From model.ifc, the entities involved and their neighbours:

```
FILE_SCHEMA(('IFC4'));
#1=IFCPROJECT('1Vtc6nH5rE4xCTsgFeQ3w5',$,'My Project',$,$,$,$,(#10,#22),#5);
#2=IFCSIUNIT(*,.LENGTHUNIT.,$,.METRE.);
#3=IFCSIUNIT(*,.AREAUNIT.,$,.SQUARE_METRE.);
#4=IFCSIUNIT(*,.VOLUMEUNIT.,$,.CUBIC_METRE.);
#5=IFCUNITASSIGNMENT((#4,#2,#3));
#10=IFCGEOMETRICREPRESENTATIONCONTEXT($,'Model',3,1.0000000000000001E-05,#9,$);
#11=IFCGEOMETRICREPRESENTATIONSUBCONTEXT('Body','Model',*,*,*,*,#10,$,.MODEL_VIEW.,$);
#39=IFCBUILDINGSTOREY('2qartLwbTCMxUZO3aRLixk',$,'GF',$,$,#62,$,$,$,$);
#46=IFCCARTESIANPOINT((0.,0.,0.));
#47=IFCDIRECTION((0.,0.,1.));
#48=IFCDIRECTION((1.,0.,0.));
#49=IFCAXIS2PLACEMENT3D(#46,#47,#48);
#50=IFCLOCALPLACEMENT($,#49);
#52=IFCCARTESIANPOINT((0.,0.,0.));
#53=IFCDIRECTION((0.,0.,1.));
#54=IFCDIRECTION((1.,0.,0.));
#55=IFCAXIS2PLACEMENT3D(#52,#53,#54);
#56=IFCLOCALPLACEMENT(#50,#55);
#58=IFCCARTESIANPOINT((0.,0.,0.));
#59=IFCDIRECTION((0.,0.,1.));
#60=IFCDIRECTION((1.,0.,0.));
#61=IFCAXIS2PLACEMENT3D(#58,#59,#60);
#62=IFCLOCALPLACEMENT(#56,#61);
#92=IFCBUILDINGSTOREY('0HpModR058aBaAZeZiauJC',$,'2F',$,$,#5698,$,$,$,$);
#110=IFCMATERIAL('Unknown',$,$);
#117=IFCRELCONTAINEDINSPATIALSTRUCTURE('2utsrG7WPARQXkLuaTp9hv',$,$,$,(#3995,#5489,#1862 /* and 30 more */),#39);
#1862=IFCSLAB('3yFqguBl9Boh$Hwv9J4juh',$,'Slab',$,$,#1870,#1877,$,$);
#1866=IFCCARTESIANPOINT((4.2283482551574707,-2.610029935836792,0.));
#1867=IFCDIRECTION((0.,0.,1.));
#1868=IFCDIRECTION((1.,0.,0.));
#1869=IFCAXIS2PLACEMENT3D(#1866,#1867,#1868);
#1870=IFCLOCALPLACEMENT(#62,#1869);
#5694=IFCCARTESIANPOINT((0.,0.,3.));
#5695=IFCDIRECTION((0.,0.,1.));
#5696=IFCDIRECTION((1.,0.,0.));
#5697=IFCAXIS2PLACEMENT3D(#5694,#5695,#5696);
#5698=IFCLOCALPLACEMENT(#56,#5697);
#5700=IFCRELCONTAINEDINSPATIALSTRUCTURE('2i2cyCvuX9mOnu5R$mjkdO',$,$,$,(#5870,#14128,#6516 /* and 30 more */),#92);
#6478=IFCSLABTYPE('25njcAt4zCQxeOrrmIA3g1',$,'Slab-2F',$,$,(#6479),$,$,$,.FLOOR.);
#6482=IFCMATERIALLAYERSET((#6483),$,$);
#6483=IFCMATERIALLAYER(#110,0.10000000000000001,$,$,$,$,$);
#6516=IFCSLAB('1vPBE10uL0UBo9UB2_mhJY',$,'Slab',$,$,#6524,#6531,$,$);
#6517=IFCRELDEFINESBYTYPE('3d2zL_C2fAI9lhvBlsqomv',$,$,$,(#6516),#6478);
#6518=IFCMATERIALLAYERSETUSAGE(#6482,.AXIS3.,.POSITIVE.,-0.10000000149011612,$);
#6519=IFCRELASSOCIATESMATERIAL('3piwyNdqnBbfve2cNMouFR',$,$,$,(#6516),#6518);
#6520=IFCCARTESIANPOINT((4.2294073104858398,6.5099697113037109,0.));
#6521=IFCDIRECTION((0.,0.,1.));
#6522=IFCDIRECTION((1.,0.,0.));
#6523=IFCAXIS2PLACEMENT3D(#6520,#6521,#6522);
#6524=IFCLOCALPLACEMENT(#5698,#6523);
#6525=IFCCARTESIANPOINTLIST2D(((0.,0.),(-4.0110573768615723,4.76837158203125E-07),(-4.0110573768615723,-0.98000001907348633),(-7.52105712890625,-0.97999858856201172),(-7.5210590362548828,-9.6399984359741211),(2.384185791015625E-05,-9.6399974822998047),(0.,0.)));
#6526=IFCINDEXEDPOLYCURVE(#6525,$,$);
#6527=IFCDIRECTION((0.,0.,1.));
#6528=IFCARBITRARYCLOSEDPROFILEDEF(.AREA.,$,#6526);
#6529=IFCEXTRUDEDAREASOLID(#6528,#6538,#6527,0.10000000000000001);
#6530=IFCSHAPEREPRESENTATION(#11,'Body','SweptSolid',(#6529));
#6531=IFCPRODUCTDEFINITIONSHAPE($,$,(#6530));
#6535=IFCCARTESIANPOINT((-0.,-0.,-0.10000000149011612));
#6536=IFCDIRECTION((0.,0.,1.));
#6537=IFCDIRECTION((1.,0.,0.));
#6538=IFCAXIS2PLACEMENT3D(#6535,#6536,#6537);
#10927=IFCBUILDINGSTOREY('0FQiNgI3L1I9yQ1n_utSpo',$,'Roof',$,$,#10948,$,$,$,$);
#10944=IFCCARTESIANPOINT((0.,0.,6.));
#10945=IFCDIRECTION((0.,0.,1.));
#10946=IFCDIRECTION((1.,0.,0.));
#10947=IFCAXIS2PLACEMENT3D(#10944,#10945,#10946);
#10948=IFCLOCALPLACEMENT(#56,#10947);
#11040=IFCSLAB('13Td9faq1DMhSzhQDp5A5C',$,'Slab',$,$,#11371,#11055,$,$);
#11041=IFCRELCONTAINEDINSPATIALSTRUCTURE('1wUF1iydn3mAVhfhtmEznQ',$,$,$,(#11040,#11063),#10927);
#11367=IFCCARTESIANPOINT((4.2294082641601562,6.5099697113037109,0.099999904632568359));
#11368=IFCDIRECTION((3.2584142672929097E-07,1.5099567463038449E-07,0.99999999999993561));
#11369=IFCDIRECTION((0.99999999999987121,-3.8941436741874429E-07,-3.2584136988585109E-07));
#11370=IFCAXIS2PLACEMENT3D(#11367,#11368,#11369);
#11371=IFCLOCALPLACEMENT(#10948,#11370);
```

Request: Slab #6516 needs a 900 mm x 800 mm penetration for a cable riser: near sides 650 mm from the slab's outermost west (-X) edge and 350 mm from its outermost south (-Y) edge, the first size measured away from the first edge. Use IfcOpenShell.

```python
import numpy as np
import ifcopenshell
import ifcopenshell.api.feature
import ifcopenshell.api.geometry
import ifcopenshell.api.root
import ifcopenshell.geom
import ifcopenshell.util.placement
import ifcopenshell.util.representation
import ifcopenshell.util.shape
import ifcopenshell.util.unit

model = ifcopenshell.open("model.ifc")
unit_scale = ifcopenshell.util.unit.calculate_unit_scale(model)
settings = ifcopenshell.geom.settings()


def volume(element):
    """Net volume in cubic metres, openings subtracted."""
    shape = ifcopenshell.geom.create_shape(settings, element)
    return ifcopenshell.util.shape.get_volume(shape.geometry)


slab = model.by_guid("1vPBE10uL0UBo9UB2_mhJY")
before = volume(slab)

# Extent in the slab's own axes, in metres. The edges named are its -X and -Y sides.
slab_shape = ifcopenshell.geom.create_shape(settings, slab)
vertices = ifcopenshell.util.shape.get_vertices(slab_shape.geometry)
x_min, y_min, bottom = vertices.min(axis=0)
top = vertices[:, 2].max()

opening = ifcopenshell.api.root.create_entity(model, ifc_class="IfcOpeningElement", name="Cable riser opening", predefined_type="OPENING")
context = ifcopenshell.util.representation.get_context(model, "Model", "Body", "MODEL_VIEW")
width, depth = 0.9, 0.8
outline = [(0.0, 0.0), (width, 0.0), (width, depth), (0.0, depth), (0.0, 0.0)]
# Overshoot both faces by 50 mm so the cut is clean.
shape = ifcopenshell.api.geometry.add_slab_representation(
    model, context=context, depth=top - bottom + 0.1, polyline=outline
)
ifcopenshell.api.geometry.assign_representation(model, product=opening, representation=shape)

matrix = ifcopenshell.util.placement.get_local_placement(slab.ObjectPlacement)
matrix[:, 3] = matrix @ np.append(np.array([x_min + 0.65, y_min + 0.35, bottom - 0.05]) / unit_scale, 1.0)
ifcopenshell.api.geometry.edit_object_placement(model, product=opening, matrix=matrix, is_si=False)
ifcopenshell.api.feature.add_feature(model, feature=opening, element=slab)

after = volume(slab)

print(f"slab volume {before:.3f} -> {after:.3f} m3")

model.write("model_updated.ifc")
```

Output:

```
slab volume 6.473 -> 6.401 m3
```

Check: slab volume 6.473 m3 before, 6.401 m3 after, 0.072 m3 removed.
